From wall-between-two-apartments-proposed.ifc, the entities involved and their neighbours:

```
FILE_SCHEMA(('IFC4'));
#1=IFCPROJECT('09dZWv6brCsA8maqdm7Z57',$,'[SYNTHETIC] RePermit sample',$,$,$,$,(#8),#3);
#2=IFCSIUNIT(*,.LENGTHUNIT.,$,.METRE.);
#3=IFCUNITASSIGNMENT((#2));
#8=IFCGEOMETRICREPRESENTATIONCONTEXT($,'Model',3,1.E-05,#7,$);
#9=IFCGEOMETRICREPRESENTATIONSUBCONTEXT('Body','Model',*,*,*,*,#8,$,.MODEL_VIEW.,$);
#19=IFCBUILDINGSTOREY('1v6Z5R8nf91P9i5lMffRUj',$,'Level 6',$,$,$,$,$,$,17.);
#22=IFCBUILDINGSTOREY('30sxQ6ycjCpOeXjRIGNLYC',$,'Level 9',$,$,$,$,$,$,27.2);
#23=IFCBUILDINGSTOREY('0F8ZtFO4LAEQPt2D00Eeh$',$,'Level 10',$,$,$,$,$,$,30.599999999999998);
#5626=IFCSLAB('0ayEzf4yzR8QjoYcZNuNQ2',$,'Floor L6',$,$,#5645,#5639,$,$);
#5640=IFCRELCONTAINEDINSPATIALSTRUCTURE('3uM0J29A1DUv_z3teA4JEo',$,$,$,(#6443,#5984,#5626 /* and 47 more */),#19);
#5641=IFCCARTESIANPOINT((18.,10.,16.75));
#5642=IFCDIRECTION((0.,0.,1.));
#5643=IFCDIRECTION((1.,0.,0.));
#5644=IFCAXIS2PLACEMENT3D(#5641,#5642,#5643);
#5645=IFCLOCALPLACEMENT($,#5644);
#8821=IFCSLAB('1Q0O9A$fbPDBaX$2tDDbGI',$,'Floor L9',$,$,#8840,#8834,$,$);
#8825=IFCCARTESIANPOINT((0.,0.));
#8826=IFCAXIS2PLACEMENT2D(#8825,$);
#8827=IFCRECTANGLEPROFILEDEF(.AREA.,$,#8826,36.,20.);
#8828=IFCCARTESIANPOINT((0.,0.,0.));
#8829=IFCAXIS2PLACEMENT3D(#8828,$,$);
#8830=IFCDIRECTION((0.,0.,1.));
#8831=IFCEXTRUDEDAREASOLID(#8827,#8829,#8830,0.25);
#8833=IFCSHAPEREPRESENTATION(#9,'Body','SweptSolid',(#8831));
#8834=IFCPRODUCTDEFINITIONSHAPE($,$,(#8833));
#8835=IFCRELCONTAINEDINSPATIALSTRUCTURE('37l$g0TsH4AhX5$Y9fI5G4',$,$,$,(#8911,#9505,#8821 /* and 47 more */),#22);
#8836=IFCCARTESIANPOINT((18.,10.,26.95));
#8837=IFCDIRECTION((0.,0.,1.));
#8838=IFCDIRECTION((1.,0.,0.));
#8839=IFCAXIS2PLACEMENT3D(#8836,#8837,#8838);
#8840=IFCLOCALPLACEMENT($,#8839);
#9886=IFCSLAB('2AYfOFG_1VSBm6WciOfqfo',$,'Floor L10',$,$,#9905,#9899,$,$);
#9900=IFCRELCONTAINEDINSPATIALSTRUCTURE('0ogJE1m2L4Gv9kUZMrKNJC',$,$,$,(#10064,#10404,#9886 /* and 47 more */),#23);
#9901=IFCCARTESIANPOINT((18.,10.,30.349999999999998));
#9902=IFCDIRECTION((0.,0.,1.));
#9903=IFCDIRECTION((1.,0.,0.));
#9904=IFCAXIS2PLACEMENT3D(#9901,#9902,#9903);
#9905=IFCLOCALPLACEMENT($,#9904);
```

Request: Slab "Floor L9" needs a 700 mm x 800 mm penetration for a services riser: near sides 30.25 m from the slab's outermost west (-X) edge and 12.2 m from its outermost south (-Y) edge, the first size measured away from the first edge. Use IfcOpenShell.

```python
import numpy as np
import ifcopenshell
import ifcopenshell.api.feature
import ifcopenshell.api.geometry
import ifcopenshell.api.root
import ifcopenshell.geom
import ifcopenshell.util.placement
import ifcopenshell.util.representation
import ifcopenshell.util.shape
import ifcopenshell.util.unit

model = ifcopenshell.open("wall-between-two-apartments-proposed.ifc")
unit_scale = ifcopenshell.util.unit.calculate_unit_scale(model)
settings = ifcopenshell.geom.settings()


def volume(element):
    """Net volume in cubic metres, openings subtracted."""
    shape = ifcopenshell.geom.create_shape(settings, element)
    return ifcopenshell.util.shape.get_volume(shape.geometry)


slab = model.by_guid("1Q0O9A$fbPDBaX$2tDDbGI")
before = volume(slab)

# Extent in the slab's own axes, in metres. The edges named are its -X and -Y sides.
slab_shape = ifcopenshell.geom.create_shape(settings, slab)
vertices = ifcopenshell.util.shape.get_vertices(slab_shape.geometry)
x_min, y_min, bottom = vertices.min(axis=0)
top = vertices[:, 2].max()

opening = ifcopenshell.api.root.create_entity(model, ifc_class="IfcOpeningElement", name="Services riser opening", predefined_type="OPENING")
context = ifcopenshell.util.representation.get_context(model, "Model", "Body", "MODEL_VIEW")
width, depth = 0.7, 0.8
outline = [(0.0, 0.0), (width, 0.0), (width, depth), (0.0, depth), (0.0, 0.0)]
# Overshoot both faces by 50 mm so the cut is clean.
shape = ifcopenshell.api.geometry.add_slab_representation(
    model, context=context, depth=top - bottom + 0.1, polyline=outline
)
ifcopenshell.api.geometry.assign_representation(model, product=opening, representation=shape)

matrix = ifcopenshell.util.placement.get_local_placement(slab.ObjectPlacement)
matrix[:, 3] = matrix @ np.append(np.array([x_min + 30.25, y_min + 12.2, bottom - 0.05]) / unit_scale, 1.0)
ifcopenshell.api.geometry.edit_object_placement(model, product=opening, matrix=matrix, is_si=False)
ifcopenshell.api.feature.add_feature(model, feature=opening, element=slab)

after = volume(slab)

print(f"slab volume {before:.3f} -> {after:.3f} m3")

model.write("wall-between-two-apartments-proposed_edited.ifc")
```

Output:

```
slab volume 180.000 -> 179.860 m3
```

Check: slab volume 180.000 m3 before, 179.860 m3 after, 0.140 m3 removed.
